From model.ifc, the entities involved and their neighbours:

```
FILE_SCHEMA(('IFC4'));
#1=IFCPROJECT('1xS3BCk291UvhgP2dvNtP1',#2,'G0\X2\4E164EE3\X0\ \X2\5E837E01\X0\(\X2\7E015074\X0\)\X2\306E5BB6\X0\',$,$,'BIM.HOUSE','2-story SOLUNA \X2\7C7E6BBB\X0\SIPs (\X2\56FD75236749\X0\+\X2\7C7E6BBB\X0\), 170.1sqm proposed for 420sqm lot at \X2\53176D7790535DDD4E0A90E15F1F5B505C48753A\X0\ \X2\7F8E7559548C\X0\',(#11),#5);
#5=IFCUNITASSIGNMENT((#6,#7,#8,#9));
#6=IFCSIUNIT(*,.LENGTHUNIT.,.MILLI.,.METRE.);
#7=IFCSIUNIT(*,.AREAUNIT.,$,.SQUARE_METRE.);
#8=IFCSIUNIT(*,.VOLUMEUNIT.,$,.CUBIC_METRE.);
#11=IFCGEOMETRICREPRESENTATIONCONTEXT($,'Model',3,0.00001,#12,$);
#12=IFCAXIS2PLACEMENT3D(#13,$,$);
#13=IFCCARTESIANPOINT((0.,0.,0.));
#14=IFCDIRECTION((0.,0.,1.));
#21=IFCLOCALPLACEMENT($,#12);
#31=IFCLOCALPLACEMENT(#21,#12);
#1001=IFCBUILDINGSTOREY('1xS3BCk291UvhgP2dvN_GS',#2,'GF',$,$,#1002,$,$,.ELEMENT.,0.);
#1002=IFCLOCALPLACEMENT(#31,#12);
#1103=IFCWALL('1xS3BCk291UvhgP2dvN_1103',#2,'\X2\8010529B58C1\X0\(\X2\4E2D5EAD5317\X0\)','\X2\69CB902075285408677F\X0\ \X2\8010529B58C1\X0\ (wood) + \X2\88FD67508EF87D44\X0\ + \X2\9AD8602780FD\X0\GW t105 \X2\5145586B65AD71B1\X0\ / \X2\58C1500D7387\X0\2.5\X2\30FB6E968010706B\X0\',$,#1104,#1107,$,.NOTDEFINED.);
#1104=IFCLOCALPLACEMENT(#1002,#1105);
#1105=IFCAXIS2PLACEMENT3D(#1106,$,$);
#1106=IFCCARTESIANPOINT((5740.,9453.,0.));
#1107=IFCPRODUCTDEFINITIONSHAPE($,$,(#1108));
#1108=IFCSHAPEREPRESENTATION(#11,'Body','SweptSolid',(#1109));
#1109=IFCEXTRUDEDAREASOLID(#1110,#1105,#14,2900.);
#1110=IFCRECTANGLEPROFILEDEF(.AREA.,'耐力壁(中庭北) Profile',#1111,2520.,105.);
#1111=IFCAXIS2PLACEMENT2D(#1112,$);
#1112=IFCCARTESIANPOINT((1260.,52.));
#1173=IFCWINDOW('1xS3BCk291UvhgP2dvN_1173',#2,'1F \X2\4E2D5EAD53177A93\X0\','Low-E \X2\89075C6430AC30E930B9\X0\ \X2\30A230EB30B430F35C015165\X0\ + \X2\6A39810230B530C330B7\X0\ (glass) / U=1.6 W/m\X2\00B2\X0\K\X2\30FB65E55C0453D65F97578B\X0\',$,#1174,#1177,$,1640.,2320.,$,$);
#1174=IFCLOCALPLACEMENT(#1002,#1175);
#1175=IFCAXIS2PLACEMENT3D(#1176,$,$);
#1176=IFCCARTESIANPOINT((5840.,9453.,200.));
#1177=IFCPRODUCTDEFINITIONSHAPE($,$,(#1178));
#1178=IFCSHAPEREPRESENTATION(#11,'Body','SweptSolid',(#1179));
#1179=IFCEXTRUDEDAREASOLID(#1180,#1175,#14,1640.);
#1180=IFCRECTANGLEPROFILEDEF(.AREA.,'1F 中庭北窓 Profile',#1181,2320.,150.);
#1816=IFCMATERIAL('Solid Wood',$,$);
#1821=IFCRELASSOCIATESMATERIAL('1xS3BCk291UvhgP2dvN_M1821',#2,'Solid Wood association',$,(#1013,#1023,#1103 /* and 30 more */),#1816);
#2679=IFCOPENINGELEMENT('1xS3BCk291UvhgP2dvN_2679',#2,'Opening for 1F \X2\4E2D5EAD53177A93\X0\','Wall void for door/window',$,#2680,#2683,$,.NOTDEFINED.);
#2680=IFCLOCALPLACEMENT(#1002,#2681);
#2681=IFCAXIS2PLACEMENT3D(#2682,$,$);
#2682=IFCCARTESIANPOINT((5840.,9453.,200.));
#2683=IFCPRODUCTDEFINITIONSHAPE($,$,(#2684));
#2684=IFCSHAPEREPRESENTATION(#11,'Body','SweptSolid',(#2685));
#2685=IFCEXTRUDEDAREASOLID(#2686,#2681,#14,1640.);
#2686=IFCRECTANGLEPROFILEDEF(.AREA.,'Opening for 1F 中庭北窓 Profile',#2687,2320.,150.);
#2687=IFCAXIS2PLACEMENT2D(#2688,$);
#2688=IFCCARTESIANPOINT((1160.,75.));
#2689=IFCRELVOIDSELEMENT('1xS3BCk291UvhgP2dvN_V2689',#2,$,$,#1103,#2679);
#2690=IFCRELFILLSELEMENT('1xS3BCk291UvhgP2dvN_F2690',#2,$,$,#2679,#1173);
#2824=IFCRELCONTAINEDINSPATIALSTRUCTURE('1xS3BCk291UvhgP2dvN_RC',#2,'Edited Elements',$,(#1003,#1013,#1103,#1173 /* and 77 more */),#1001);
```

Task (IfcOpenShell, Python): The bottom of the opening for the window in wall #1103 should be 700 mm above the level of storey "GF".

```python
import numpy as np
import ifcopenshell
import ifcopenshell.api.geometry
import ifcopenshell.geom
import ifcopenshell.util.element
import ifcopenshell.util.placement
import ifcopenshell.util.shape
import ifcopenshell.util.unit

model = ifcopenshell.open("model.ifc")
unit_scale = ifcopenshell.util.unit.calculate_unit_scale(model)

window = model.by_guid("1xS3BCk291UvhgP2dvN_1173")
opening = window.FillsVoids[0].RelatingOpeningElement
storey = ifcopenshell.util.element.get_container(window, ifc_class="IfcBuildingStorey")
level = ifcopenshell.util.placement.get_local_placement(storey.ObjectPlacement)[2, 3]

# The opening's origin need not be at the sill, so measure its lowest point.
shape = ifcopenshell.geom.create_shape(ifcopenshell.geom.settings(), opening)
bottom = ifcopenshell.util.shape.get_shape_bottom_elevation(shape, shape.geometry) / unit_scale
dz = level + 0.7 / unit_scale - bottom

shift = np.array([0.0, 0.0, dz])
# The window is not placed relative to its opening, so move both.
for product in (opening, window):
    matrix = ifcopenshell.util.placement.get_local_placement(product.ObjectPlacement)
    matrix[:3, 3] += shift
    ifcopenshell.api.geometry.edit_object_placement(model, product=product, matrix=matrix, is_si=False)

print(f"moved by {dz * unit_scale:+.3f} m")

model.write("model_updated.ifc")
```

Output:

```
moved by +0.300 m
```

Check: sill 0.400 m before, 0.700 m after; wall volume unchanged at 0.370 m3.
